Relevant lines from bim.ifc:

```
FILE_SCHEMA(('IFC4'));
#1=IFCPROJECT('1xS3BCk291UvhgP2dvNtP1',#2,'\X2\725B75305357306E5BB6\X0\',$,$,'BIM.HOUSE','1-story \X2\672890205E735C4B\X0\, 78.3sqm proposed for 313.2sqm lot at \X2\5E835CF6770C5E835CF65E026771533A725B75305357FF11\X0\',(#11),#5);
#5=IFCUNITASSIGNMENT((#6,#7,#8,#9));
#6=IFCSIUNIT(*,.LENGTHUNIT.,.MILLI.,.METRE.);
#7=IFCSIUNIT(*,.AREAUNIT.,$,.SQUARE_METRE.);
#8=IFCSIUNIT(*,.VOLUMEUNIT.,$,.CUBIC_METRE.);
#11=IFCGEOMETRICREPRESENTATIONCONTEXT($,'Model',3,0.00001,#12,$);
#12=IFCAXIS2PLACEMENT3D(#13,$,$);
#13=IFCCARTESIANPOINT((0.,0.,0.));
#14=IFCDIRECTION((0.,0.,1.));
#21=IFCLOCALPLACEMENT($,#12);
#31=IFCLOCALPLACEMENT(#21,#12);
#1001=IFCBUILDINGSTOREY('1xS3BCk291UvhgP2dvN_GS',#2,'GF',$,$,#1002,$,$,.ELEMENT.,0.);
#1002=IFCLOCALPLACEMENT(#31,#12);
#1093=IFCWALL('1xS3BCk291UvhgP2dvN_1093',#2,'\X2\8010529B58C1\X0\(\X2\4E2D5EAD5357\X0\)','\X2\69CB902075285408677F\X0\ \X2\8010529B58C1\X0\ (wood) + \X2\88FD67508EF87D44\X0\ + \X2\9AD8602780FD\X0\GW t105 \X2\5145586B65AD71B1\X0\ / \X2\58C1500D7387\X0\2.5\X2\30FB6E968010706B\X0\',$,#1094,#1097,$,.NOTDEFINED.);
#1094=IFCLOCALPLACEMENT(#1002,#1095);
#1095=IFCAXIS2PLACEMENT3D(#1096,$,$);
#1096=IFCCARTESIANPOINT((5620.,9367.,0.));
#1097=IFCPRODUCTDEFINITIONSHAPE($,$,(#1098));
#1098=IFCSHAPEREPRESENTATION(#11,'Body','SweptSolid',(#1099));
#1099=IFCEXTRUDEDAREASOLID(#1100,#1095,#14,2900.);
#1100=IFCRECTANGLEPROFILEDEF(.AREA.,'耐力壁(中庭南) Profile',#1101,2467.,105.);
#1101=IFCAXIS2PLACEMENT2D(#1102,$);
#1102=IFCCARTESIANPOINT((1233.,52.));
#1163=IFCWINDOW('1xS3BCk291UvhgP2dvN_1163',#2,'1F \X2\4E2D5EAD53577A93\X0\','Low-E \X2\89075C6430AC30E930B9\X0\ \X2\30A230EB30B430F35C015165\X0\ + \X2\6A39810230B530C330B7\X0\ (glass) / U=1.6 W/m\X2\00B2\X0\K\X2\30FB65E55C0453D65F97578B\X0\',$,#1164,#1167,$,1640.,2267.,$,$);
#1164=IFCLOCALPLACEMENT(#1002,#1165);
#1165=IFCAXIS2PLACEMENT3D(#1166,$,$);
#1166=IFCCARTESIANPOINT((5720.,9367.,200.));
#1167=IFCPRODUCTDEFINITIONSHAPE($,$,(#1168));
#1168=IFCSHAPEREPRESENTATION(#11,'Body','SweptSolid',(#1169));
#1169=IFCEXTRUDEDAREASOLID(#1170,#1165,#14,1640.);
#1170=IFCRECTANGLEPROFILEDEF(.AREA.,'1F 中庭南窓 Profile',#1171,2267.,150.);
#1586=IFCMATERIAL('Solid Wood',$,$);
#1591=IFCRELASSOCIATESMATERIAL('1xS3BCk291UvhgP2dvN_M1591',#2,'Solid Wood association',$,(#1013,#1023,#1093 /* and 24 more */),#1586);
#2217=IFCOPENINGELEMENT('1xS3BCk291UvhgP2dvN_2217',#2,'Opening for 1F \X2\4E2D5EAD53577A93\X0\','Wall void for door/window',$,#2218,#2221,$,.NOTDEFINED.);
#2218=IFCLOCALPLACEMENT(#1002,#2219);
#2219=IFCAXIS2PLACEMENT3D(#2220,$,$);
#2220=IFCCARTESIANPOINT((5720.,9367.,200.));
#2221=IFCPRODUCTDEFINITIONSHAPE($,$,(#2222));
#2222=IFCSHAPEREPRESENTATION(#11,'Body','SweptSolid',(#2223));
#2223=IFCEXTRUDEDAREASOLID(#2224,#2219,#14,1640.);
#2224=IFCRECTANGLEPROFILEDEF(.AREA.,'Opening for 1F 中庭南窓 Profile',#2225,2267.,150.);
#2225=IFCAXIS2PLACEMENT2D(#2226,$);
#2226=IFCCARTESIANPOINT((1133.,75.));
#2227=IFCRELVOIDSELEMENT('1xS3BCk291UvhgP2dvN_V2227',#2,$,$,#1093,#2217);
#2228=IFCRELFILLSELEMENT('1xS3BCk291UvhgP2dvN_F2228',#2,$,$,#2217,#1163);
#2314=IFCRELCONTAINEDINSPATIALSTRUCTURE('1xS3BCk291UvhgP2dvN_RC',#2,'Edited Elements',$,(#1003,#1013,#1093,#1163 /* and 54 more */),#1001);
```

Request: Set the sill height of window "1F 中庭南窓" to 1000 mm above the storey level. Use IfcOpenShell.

```python
import numpy as np
import ifcopenshell
import ifcopenshell.api.geometry
import ifcopenshell.geom
import ifcopenshell.util.element
import ifcopenshell.util.placement
import ifcopenshell.util.shape
import ifcopenshell.util.unit

model = ifcopenshell.open("bim.ifc")
unit_scale = ifcopenshell.util.unit.calculate_unit_scale(model)

window = model.by_guid("1xS3BCk291UvhgP2dvN_1163")
opening = window.FillsVoids[0].RelatingOpeningElement
storey = ifcopenshell.util.element.get_container(window, ifc_class="IfcBuildingStorey")
level = ifcopenshell.util.placement.get_local_placement(storey.ObjectPlacement)[2, 3]

# The opening's origin need not be at the sill, so measure its lowest point.
shape = ifcopenshell.geom.create_shape(ifcopenshell.geom.settings(), opening)
bottom = ifcopenshell.util.shape.get_shape_bottom_elevation(shape, shape.geometry) / unit_scale
dz = level + 1 / unit_scale - bottom

shift = np.array([0.0, 0.0, dz])
# The window is not placed relative to its opening, so move both.
for product in (opening, window):
    matrix = ifcopenshell.util.placement.get_local_placement(product.ObjectPlacement)
    matrix[:3, 3] += shift
    ifcopenshell.api.geometry.edit_object_placement(model, product=product, matrix=matrix, is_si=False)

print(f"moved by {dz * unit_scale:+.3f} m")

model.write("bim_v2.ifc")
```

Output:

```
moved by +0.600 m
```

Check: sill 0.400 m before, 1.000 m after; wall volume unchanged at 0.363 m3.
